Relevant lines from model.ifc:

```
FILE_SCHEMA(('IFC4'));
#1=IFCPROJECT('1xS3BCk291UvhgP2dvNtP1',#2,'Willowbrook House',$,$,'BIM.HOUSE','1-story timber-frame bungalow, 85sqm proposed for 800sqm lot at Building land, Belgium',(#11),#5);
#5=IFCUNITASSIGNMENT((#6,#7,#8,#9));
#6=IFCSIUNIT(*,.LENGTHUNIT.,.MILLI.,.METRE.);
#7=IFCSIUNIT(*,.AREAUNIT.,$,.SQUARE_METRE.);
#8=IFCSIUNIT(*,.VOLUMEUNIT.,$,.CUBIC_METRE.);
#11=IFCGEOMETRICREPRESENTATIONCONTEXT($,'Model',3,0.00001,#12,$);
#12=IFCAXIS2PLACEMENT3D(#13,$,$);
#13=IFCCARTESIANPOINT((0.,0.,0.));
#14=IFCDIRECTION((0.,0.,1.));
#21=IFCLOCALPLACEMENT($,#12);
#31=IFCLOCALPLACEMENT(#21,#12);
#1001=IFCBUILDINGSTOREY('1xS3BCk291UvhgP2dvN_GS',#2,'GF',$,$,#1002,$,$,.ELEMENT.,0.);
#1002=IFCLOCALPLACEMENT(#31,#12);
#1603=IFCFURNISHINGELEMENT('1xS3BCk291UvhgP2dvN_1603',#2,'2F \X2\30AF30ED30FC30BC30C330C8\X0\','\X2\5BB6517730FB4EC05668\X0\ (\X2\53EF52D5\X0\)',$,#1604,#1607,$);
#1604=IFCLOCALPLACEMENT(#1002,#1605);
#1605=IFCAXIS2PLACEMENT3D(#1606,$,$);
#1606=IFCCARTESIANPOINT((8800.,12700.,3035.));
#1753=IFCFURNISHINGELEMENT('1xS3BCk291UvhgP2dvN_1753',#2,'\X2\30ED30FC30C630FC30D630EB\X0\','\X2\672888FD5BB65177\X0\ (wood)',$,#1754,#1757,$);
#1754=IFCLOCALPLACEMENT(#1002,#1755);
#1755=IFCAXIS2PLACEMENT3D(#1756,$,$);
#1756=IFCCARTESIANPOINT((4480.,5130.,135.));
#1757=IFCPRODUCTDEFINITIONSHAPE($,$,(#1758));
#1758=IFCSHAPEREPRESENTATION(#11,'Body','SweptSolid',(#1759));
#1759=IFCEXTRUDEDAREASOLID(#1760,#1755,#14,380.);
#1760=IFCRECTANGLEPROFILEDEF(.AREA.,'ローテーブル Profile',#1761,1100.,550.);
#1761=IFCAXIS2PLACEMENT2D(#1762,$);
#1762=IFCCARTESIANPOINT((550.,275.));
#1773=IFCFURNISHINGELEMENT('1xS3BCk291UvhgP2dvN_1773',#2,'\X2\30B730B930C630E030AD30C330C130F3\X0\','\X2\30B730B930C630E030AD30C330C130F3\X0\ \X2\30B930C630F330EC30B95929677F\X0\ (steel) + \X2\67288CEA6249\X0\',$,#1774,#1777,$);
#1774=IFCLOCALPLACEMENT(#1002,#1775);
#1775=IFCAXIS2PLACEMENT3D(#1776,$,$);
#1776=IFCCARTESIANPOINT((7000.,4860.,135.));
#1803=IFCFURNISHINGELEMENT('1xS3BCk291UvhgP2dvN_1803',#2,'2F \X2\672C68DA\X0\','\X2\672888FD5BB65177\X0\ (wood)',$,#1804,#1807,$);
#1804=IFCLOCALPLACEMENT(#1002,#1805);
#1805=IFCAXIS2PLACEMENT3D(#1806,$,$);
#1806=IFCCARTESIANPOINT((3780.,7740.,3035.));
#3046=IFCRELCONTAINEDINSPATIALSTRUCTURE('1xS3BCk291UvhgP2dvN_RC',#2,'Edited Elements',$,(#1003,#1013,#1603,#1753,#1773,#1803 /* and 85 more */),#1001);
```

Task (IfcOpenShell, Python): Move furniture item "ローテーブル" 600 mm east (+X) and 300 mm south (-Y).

```python
import ifcopenshell
import ifcopenshell.api.geometry
import ifcopenshell.util.placement

model = ifcopenshell.open("model.ifc")

item = model.by_guid("1xS3BCk291UvhgP2dvN_1753")
matrix = ifcopenshell.util.placement.get_local_placement(item.ObjectPlacement)
matrix[0, 3] += 600.0
matrix[1, 3] -= 300.0
ifcopenshell.api.geometry.edit_object_placement(model, product=item, matrix=matrix, is_si=False)

print(ifcopenshell.util.placement.get_local_placement(item.ObjectPlacement).round(3) + 0.0)

model.write("model_v2.ifc")
```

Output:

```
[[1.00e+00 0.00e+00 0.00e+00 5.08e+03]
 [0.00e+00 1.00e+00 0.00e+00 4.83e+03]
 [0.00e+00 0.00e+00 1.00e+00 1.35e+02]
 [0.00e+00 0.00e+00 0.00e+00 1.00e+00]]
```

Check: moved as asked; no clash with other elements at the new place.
